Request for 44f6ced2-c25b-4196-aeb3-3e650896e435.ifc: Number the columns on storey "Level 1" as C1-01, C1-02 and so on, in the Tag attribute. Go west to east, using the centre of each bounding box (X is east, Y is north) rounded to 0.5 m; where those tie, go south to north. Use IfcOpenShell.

First a look at what the model holds.

```python
import ifcopenshell
import ifcopenshell.util.element
import ifcopenshell.util.placement

model = ifcopenshell.open("44f6ced2-c25b-4196-aeb3-3e650896e435.ifc")
print(model.schema)
storey = next(s for s in model.by_type("IfcBuildingStorey") if s.Name == "Level 1")
columns = [e for e in ifcopenshell.util.element.get_decomposition(storey) if e.is_a("IfcColumn")]
for e in sorted(columns, key=lambda e: e.id()):
    origin = ifcopenshell.util.placement.get_local_placement(e.ObjectPlacement)[:3, 3]
    print(e.id(), e.Tag, e.Name, origin.round(2) + 0.0, sep=" | ")
```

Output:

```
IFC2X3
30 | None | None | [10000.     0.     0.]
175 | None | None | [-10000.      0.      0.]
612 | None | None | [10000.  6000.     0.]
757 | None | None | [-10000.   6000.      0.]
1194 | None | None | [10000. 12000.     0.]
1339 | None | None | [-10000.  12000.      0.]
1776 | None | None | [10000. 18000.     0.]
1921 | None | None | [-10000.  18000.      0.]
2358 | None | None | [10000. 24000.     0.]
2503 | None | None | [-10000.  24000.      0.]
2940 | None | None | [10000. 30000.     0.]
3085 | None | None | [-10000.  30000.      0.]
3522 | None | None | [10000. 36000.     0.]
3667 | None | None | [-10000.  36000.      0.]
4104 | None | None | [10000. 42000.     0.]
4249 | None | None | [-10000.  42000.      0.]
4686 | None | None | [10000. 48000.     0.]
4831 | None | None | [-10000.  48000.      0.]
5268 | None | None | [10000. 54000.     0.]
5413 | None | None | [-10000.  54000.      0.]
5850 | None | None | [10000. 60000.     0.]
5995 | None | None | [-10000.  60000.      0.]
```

```python
import ifcopenshell
import ifcopenshell.geom
import ifcopenshell.util.element
import ifcopenshell.util.shape

model = ifcopenshell.open("44f6ced2-c25b-4196-aeb3-3e650896e435.ifc")
settings = ifcopenshell.geom.settings()
settings.set("use-world-coords", True)


def centre(element):
    shape = ifcopenshell.geom.create_shape(settings, element)
    return ifcopenshell.util.shape.get_bbox_centroid(shape.geometry)


storey = next(s for s in model.by_type("IfcBuildingStorey") if s.Name == "Level 1")
columns = [e for e in ifcopenshell.util.element.get_decomposition(storey) if e.is_a("IfcColumn")]

# Insertion points can sit at a corner or the storey origin, so sort by the geometry (in metres).
centres = {e: centre(e) for e in columns}
columns.sort(key=lambda e: (round(centres[e][0] / 0.5), centres[e][1]))

for i, e in enumerate(columns, start=1):
    number = f"C1-{i:02d}"
    e.Tag = number
    print(e.id(), number)

model.write("44f6ced2-c25b-4196-aeb3-3e650896e435_edited.ifc")
```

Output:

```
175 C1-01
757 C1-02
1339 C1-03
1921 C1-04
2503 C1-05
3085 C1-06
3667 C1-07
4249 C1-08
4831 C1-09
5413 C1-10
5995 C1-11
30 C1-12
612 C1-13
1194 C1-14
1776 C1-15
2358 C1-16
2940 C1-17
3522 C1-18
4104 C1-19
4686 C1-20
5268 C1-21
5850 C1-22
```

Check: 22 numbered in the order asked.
